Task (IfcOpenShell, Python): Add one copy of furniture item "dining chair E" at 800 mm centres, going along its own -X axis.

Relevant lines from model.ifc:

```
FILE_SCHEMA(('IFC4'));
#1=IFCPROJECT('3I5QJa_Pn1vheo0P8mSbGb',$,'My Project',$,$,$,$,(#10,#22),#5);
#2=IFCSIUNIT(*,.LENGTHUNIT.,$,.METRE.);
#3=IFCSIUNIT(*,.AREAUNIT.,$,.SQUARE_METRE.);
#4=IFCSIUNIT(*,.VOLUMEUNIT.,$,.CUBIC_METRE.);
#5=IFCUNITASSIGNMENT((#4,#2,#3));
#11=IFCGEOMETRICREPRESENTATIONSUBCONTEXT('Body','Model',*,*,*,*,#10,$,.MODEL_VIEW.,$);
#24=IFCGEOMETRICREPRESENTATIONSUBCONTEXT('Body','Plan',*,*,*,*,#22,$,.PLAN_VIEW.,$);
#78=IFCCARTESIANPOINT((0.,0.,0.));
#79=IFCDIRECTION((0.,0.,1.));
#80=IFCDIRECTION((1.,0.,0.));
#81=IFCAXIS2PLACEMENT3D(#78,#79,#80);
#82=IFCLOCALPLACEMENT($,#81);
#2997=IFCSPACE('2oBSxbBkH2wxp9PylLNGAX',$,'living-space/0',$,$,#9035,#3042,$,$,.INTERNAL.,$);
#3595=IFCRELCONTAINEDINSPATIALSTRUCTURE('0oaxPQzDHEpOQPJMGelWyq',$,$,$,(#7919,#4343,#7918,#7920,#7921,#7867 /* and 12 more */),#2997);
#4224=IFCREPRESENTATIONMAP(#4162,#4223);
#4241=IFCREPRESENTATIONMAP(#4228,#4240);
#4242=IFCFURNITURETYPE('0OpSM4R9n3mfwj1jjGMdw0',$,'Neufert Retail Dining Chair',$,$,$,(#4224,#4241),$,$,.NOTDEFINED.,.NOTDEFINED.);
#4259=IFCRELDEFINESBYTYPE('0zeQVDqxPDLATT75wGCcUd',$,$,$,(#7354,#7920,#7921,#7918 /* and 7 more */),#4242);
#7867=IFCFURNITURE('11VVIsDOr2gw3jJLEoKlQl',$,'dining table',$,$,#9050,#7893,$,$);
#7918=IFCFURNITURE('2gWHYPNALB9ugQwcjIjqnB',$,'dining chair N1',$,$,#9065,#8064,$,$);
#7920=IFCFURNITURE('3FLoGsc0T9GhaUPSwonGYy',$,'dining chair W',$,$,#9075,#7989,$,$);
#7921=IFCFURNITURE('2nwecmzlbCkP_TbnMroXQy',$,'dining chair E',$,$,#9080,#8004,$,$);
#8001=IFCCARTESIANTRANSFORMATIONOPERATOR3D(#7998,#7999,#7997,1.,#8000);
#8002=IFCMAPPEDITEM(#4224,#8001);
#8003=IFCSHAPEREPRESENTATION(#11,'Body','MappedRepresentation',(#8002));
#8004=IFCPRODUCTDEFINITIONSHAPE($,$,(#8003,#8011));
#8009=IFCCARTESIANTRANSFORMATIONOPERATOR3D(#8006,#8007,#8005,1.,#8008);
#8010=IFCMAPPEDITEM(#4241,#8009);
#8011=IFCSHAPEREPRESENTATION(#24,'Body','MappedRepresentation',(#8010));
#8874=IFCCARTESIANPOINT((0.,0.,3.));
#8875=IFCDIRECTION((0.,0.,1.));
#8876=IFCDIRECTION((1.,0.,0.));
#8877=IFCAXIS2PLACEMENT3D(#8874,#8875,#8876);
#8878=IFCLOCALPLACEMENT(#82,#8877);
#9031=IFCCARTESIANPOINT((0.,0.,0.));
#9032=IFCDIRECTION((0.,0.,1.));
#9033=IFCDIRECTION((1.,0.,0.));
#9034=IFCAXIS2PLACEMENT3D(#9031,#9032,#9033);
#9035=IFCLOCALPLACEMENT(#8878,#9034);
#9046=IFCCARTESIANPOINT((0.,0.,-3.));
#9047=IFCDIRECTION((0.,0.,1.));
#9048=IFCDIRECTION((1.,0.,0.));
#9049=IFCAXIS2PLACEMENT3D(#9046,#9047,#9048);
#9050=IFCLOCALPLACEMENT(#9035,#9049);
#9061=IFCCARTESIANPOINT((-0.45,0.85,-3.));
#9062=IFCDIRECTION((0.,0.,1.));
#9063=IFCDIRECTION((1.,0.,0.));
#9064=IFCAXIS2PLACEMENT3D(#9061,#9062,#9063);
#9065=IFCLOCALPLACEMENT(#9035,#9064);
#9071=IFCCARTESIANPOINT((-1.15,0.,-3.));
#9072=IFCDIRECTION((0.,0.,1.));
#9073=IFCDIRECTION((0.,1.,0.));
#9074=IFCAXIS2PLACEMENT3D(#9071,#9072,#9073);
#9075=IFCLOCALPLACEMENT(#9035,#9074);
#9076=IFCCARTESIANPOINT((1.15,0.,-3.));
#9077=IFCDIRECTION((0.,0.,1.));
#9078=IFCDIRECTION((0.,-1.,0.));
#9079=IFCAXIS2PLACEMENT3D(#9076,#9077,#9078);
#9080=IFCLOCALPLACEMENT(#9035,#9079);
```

```python
import ifcopenshell
import ifcopenshell.api.geometry
import ifcopenshell.api.root
import ifcopenshell.util.element
import ifcopenshell.util.placement
import ifcopenshell.util.unit

model = ifcopenshell.open("model.ifc")
unit_scale = ifcopenshell.util.unit.calculate_unit_scale(model)

source = model.by_guid("2nwecmzlbCkP_TbnMroXQy")
base = ifcopenshell.util.placement.get_local_placement(source.ObjectPlacement)
step = -base[:3, 0] * 0.8 / unit_scale

for i in range(1, 2):
    copy = ifcopenshell.api.root.copy_class(model, product=source)
    copy.Representation = ifcopenshell.util.element.copy_deep(
        model, source.Representation, exclude=["IfcGeometricRepresentationContext", "IfcRepresentationMap"]
    )
    matrix = base.copy()
    matrix[:3, 3] += i * step
    print("added at", matrix[:3, 3].round(3) + 0.0)
    ifcopenshell.api.geometry.edit_object_placement(model, product=copy, matrix=matrix, is_si=False)

model.write("model_edited.ifc")
```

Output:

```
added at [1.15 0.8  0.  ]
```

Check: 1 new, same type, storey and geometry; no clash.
